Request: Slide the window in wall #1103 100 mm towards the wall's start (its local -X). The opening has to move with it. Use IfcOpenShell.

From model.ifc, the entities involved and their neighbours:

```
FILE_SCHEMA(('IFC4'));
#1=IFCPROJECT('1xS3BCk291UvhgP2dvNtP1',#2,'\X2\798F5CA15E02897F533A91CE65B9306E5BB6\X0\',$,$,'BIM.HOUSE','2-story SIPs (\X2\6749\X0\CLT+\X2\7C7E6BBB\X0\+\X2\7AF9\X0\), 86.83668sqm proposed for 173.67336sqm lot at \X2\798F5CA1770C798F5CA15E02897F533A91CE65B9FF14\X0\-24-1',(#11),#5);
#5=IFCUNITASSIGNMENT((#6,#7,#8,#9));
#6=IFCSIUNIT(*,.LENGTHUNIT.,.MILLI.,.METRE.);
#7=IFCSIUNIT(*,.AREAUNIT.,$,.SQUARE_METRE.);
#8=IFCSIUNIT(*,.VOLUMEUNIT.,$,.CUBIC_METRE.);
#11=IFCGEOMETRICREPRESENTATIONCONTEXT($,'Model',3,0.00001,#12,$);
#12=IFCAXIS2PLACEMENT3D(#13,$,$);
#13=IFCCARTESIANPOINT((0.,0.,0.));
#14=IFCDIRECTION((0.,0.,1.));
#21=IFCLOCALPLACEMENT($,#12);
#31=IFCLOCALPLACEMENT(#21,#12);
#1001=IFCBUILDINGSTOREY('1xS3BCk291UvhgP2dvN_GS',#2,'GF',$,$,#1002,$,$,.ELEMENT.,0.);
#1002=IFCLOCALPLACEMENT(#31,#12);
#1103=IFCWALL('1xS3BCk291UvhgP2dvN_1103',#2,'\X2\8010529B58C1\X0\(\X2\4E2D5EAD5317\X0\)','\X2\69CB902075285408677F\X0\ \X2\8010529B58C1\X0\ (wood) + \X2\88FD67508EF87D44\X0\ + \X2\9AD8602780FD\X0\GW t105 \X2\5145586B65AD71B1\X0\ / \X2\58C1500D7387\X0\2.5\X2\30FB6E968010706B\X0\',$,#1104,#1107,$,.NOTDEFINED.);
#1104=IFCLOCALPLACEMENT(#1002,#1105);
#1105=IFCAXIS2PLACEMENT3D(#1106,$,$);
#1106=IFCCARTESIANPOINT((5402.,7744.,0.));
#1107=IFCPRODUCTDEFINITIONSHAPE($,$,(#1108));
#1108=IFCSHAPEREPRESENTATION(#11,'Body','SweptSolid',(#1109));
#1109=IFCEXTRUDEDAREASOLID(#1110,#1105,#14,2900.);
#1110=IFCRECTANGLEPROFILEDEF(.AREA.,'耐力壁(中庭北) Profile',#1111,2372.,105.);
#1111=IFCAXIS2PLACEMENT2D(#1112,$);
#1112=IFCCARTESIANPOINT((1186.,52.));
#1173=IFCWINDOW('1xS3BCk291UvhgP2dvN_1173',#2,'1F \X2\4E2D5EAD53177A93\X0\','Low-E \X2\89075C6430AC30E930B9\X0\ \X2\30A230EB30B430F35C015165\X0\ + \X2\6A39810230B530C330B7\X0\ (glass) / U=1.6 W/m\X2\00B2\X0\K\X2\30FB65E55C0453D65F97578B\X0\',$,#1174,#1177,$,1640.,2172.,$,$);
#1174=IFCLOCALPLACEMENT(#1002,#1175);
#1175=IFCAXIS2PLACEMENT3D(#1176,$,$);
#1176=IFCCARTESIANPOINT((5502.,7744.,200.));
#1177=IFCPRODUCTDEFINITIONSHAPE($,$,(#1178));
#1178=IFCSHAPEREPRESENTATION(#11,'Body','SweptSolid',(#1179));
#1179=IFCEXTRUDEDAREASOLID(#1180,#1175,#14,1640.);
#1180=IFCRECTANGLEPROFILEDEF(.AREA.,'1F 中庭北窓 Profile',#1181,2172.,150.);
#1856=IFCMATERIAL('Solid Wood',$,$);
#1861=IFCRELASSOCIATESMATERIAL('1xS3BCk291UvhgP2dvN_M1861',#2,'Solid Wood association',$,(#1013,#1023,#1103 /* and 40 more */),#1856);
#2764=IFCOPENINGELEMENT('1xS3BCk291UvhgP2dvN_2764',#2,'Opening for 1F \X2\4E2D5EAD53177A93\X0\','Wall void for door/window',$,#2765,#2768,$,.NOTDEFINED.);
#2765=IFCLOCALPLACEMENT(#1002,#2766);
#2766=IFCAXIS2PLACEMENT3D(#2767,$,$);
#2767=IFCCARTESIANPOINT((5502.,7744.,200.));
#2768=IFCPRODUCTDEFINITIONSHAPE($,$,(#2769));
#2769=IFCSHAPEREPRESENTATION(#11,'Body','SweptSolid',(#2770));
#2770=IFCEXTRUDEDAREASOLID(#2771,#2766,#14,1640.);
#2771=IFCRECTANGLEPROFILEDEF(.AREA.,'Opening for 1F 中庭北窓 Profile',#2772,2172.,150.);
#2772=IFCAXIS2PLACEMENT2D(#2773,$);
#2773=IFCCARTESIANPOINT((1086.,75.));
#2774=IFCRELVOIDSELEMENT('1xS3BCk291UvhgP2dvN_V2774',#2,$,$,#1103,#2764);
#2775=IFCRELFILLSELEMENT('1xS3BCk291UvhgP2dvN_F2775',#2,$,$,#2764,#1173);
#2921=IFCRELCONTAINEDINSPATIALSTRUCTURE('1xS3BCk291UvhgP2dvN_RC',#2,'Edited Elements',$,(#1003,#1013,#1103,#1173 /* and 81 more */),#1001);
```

```python
import ifcopenshell
import ifcopenshell.api.geometry
import ifcopenshell.util.placement
import ifcopenshell.util.unit

model = ifcopenshell.open("model.ifc")
unit_scale = ifcopenshell.util.unit.calculate_unit_scale(model)

window = model.by_guid("1xS3BCk291UvhgP2dvN_1173")
opening = window.FillsVoids[0].RelatingOpeningElement
wall = opening.VoidsElements[0].RelatingBuildingElement

wall_matrix = ifcopenshell.util.placement.get_local_placement(wall.ObjectPlacement)
shift = wall_matrix[:3, 0] * -0.1 / unit_scale
before = ifcopenshell.util.placement.get_local_placement(window.ObjectPlacement)[:3, 3].copy()

# The window is not placed relative to its opening, so move both.
for product in (opening, window):
    matrix = ifcopenshell.util.placement.get_local_placement(product.ObjectPlacement)
    matrix[:3, 3] += shift
    ifcopenshell.api.geometry.edit_object_placement(model, product=product, matrix=matrix, is_si=False)

after = ifcopenshell.util.placement.get_local_placement(window.ObjectPlacement)[:3, 3]
print("window moved by", (after - before).round(3) + 0.0)

model.write("model_edited.ifc")
```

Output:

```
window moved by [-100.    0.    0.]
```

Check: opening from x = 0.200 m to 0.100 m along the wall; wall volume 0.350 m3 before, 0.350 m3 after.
